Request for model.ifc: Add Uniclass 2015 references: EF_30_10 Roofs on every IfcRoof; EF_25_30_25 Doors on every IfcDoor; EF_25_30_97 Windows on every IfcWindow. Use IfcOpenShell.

First a look at what the model holds.

```python
import ifcopenshell

model = ifcopenshell.open("model.ifc")
print(model.schema)
print("classifications:", [c.Name for c in model.by_type("IfcClassification")])
for ifc_class in ("IfcDoor", "IfcRoof", "IfcStair", "IfcWall", "IfcWindow"):
    print(ifc_class, len(model.by_type(ifc_class)))
```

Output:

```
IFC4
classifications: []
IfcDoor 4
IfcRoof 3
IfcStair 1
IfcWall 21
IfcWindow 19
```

```python
import ifcopenshell
import ifcopenshell.api.classification

model = ifcopenshell.open("model.ifc")

system = ifcopenshell.api.classification.add_classification(model, classification="Uniclass 2015")

codes = {
    "IfcRoof": ("EF_30_10", "Roofs"),
    "IfcDoor": ("EF_25_30_25", "Doors"),
    "IfcWindow": ("EF_25_30_97", "Windows"),
}
for ifc_class, (code, name) in codes.items():
    products = model.by_type(ifc_class)
    ifcopenshell.api.classification.add_reference(
        model, products=products, classification=system, identification=code, name=name
    )
    print(code, len(products))

model.write("model_updated.ifc")
```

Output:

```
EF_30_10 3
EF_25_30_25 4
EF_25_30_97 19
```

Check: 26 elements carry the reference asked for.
